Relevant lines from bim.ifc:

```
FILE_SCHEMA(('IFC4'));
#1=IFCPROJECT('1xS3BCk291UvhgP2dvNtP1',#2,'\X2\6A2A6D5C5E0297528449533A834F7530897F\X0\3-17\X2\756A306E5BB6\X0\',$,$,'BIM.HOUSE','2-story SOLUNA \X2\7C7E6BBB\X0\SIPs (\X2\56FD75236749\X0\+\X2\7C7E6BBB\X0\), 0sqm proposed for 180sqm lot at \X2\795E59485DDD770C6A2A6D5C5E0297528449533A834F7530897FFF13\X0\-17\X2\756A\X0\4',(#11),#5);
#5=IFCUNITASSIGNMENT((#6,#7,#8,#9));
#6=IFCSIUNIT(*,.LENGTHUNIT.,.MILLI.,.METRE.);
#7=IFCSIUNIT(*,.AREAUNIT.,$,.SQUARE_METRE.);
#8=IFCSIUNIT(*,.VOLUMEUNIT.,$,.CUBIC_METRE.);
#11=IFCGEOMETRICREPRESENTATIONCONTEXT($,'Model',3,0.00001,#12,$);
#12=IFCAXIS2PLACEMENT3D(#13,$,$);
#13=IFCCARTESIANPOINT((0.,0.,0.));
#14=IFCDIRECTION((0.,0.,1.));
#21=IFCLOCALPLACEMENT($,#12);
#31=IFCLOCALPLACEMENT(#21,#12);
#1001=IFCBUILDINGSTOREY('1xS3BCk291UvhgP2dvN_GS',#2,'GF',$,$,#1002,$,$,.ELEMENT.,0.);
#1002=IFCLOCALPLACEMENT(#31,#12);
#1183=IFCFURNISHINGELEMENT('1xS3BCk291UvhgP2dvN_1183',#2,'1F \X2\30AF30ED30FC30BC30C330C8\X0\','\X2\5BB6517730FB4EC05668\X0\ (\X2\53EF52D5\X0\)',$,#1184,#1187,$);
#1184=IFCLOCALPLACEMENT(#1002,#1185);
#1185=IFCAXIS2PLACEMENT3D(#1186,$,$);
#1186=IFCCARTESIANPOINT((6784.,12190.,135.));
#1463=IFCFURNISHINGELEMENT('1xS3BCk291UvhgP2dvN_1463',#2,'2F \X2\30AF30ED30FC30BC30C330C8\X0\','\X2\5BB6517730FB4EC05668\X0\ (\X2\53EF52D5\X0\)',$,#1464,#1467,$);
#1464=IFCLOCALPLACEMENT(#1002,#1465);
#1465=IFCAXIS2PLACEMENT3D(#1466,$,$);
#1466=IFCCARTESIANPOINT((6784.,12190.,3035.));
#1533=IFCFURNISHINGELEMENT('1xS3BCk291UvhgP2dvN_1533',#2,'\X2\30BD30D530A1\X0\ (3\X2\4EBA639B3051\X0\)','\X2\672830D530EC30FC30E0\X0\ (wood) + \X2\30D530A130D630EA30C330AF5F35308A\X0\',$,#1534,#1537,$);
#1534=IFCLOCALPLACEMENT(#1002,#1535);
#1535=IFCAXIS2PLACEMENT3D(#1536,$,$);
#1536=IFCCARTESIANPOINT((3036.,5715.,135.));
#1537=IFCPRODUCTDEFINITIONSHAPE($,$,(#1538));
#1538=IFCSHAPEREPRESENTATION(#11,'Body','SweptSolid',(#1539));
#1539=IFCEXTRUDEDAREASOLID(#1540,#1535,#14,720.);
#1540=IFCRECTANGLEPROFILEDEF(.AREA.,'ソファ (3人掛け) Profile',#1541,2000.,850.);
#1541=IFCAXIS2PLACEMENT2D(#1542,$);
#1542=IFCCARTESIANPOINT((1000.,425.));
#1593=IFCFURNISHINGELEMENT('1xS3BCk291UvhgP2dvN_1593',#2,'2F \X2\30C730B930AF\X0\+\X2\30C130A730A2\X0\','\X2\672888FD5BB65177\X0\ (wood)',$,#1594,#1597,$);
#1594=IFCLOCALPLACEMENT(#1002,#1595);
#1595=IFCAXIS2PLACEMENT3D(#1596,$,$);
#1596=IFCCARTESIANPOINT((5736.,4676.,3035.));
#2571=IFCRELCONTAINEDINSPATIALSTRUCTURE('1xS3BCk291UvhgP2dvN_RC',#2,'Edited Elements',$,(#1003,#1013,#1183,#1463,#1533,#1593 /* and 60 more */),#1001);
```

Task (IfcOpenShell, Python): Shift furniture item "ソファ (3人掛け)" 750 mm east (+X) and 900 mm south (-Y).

```python
import ifcopenshell
import ifcopenshell.api.geometry
import ifcopenshell.util.placement

model = ifcopenshell.open("bim.ifc")

item = model.by_guid("1xS3BCk291UvhgP2dvN_1533")
matrix = ifcopenshell.util.placement.get_local_placement(item.ObjectPlacement)
matrix[0, 3] += 750.0
matrix[1, 3] -= 900.0
ifcopenshell.api.geometry.edit_object_placement(model, product=item, matrix=matrix, is_si=False)

print(ifcopenshell.util.placement.get_local_placement(item.ObjectPlacement).round(3) + 0.0)

model.write("bim_rev.ifc")
```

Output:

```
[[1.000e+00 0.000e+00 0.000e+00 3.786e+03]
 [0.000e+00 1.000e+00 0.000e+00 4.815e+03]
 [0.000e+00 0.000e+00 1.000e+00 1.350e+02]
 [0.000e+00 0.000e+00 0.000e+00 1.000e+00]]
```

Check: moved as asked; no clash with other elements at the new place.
